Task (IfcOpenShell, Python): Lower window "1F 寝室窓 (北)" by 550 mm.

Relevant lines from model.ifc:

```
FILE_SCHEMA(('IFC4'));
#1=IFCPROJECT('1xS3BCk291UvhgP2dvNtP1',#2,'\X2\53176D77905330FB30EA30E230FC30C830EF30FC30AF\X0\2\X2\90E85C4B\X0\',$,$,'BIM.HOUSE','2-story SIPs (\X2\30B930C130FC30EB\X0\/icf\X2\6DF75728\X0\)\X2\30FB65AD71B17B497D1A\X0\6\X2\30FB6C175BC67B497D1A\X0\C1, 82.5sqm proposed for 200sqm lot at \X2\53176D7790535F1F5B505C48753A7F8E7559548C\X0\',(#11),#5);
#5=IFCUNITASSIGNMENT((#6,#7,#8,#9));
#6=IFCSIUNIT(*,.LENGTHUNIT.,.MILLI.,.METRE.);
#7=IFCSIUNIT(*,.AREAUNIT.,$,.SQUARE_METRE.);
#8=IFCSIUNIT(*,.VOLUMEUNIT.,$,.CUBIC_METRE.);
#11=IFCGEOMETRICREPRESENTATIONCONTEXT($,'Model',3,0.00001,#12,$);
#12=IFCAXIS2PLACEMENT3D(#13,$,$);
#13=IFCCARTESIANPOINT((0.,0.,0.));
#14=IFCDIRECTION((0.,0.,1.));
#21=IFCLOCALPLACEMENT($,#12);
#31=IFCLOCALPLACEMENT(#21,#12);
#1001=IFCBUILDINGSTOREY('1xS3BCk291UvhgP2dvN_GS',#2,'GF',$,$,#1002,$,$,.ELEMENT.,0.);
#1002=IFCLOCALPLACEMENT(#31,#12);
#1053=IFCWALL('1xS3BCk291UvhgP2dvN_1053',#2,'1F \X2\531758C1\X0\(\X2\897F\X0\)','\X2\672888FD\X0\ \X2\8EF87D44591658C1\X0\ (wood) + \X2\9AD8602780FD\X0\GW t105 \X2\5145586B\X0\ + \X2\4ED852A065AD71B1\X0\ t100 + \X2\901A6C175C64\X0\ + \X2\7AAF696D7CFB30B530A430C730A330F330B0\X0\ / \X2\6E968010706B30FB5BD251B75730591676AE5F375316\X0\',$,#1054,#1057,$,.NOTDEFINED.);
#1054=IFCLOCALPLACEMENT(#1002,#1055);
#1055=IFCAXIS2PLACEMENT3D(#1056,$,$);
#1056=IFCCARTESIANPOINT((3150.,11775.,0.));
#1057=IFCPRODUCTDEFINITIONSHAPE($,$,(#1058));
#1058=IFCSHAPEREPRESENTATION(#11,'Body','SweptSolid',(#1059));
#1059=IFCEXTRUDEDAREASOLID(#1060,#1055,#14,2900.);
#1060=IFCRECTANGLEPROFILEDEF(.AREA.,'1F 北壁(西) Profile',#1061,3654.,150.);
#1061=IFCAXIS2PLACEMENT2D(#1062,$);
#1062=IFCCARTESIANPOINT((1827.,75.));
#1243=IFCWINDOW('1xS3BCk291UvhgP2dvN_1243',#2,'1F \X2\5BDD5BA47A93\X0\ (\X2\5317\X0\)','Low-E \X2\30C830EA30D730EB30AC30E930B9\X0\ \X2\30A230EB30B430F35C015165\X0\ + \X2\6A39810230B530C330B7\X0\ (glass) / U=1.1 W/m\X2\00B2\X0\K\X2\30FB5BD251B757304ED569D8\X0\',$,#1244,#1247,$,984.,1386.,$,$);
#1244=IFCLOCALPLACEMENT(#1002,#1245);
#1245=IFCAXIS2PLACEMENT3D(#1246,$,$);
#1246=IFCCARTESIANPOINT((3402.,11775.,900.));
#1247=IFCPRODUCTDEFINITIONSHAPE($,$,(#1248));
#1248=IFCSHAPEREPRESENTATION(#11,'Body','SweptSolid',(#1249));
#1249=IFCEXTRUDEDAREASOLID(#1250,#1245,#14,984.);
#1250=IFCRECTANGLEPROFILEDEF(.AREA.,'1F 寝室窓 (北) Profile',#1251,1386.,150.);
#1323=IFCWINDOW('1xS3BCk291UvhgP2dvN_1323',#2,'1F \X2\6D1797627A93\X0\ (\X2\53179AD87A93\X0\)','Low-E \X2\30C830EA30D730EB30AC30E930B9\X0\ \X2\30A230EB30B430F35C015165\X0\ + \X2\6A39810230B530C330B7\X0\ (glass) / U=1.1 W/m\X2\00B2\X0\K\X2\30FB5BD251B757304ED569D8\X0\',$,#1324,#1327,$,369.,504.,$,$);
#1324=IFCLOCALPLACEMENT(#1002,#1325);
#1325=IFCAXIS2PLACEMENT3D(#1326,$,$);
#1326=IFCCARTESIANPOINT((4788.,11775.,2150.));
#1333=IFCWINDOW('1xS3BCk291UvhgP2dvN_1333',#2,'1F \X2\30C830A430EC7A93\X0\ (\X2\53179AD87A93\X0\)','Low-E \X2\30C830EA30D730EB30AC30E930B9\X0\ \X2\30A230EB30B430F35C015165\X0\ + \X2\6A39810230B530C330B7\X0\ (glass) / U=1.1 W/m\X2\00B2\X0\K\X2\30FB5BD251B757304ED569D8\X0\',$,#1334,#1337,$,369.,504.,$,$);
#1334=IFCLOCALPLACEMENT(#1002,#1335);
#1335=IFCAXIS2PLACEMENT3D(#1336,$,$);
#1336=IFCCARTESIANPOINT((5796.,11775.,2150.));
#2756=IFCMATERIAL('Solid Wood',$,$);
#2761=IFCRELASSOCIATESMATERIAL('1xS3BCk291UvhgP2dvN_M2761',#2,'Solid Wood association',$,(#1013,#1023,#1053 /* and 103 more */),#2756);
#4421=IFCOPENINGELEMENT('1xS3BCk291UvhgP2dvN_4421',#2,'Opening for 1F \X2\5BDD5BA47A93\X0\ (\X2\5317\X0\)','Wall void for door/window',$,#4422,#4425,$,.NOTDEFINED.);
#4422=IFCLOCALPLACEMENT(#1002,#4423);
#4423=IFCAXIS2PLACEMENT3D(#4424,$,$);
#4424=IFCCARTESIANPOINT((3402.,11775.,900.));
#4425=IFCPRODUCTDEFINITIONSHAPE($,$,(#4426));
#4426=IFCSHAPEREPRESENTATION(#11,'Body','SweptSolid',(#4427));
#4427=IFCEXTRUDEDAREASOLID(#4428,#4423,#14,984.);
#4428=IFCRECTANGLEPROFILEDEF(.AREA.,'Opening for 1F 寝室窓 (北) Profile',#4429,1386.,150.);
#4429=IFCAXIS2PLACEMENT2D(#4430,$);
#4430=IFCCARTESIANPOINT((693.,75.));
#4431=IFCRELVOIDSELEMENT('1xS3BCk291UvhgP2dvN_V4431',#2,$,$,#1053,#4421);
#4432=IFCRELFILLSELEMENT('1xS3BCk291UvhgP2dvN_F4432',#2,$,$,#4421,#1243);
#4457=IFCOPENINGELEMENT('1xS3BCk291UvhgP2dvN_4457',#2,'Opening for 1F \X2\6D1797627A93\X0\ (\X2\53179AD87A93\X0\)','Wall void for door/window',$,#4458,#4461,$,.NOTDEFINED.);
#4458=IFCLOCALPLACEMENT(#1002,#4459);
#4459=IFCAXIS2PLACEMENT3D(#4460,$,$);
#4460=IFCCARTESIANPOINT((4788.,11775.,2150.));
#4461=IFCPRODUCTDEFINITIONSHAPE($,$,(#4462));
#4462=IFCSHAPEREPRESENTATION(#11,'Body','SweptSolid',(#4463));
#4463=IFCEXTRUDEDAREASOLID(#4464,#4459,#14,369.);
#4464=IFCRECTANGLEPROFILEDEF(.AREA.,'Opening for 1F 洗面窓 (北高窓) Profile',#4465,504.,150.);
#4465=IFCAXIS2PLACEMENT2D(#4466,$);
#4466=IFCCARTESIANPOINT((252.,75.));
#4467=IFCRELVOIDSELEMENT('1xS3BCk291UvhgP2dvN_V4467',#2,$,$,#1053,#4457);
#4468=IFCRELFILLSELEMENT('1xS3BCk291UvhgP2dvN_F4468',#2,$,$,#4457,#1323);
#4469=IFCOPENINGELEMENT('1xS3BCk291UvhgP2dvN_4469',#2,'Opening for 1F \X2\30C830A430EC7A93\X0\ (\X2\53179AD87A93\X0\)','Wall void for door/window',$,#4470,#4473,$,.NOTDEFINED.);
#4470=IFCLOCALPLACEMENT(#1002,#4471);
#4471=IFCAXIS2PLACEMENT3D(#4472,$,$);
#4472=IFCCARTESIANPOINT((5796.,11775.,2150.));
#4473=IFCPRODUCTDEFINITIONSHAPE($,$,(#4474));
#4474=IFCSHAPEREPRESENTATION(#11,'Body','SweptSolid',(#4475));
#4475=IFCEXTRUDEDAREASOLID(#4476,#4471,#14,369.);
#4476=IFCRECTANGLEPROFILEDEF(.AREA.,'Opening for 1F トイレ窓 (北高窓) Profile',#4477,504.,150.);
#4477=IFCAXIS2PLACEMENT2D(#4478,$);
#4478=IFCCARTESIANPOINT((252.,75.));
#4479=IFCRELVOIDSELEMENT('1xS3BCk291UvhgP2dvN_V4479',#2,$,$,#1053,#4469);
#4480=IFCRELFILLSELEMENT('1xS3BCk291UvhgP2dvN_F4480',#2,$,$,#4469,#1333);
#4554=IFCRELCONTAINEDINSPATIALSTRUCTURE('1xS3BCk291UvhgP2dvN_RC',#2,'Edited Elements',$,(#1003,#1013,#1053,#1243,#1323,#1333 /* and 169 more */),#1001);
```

```python
import numpy as np
import ifcopenshell
import ifcopenshell.api.geometry
import ifcopenshell.util.placement
import ifcopenshell.util.unit

model = ifcopenshell.open("model.ifc")
unit_scale = ifcopenshell.util.unit.calculate_unit_scale(model)

window = model.by_id(1243)
opening = window.FillsVoids[0].RelatingOpeningElement
dz = -0.55 / unit_scale

shift = np.array([0.0, 0.0, dz])
# The window is not placed relative to its opening, so move both.
for product in (opening, window):
    matrix = ifcopenshell.util.placement.get_local_placement(product.ObjectPlacement)
    matrix[:3, 3] += shift
    ifcopenshell.api.geometry.edit_object_placement(model, product=product, matrix=matrix, is_si=False)

print(f"moved by {dz * unit_scale:+.3f} m")

model.write("model_rev.ifc")
```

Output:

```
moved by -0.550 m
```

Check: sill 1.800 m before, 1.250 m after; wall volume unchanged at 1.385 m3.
